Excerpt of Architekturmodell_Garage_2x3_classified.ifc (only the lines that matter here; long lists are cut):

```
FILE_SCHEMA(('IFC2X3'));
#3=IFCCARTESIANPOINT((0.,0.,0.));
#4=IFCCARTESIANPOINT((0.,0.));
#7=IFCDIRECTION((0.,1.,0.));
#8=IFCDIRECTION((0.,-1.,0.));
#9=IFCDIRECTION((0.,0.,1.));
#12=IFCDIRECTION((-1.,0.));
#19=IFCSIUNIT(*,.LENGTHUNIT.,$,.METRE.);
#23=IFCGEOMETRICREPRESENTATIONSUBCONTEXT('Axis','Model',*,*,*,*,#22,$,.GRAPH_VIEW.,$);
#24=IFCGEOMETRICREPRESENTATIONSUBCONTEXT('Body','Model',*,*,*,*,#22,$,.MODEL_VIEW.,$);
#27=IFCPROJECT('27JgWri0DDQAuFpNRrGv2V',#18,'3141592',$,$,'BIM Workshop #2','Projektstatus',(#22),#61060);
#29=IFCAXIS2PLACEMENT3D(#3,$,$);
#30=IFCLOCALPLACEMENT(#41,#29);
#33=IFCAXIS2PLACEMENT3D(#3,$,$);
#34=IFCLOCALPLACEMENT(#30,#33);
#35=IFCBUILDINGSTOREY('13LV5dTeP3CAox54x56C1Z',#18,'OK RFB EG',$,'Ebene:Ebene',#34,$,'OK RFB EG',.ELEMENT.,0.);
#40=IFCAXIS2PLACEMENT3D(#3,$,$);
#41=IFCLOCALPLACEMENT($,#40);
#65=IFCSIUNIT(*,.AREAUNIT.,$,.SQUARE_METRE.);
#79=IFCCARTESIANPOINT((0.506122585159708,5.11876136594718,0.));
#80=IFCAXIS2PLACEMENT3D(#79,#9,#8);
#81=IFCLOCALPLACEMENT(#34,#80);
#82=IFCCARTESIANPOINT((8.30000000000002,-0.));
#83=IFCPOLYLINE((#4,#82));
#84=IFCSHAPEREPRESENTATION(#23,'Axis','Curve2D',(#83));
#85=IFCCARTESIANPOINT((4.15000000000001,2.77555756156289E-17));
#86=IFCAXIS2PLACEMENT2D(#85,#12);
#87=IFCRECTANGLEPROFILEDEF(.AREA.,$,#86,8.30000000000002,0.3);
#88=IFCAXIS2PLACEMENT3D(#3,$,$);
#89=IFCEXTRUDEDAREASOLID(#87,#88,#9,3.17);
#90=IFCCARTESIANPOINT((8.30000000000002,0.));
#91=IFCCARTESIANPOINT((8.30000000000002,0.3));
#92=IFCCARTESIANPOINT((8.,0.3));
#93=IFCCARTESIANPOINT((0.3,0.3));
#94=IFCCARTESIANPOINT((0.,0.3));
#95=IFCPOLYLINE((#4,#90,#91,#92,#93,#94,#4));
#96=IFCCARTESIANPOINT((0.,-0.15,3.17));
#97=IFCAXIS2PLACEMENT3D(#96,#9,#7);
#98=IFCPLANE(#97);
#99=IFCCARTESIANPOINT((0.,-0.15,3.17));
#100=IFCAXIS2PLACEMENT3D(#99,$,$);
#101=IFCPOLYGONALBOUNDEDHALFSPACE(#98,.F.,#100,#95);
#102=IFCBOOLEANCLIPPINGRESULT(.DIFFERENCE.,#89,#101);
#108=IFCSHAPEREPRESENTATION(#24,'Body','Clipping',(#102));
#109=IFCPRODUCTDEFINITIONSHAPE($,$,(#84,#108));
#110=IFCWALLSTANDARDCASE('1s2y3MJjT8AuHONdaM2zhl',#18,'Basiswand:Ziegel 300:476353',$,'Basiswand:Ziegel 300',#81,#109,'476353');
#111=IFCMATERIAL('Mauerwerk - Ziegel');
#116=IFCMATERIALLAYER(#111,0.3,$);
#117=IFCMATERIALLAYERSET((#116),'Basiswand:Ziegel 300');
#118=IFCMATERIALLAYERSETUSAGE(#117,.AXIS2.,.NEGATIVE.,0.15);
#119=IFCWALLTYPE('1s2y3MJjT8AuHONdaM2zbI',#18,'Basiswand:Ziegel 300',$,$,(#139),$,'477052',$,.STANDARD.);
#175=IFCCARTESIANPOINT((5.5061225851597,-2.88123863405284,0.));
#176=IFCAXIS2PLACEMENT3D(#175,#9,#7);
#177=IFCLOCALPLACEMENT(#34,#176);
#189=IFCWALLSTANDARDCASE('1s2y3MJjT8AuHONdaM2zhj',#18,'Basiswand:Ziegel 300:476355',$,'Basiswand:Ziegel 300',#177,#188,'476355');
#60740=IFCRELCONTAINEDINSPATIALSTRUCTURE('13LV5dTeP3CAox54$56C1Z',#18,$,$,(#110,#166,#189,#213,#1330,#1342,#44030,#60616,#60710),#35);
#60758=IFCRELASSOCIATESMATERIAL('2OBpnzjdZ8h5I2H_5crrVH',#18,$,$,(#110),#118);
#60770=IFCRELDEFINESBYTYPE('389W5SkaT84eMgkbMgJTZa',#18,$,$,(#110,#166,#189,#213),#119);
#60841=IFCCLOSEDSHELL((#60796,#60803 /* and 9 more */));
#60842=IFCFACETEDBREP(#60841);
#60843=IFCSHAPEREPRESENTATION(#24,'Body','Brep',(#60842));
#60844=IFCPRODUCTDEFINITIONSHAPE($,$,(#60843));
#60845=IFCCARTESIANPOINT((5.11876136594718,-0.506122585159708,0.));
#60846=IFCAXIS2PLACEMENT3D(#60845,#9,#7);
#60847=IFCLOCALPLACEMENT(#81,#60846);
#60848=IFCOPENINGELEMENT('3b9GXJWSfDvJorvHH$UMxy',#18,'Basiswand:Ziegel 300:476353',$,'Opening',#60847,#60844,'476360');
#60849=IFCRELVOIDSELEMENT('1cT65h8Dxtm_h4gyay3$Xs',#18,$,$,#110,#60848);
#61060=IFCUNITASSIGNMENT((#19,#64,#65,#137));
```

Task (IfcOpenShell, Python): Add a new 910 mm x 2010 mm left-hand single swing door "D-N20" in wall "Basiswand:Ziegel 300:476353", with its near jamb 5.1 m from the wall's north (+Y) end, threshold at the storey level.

```python
import numpy as np
import ifcopenshell
import ifcopenshell.api.feature
import ifcopenshell.api.geometry
import ifcopenshell.api.root
import ifcopenshell.api.spatial
import ifcopenshell.api.type
import ifcopenshell.geom
import ifcopenshell.util.element
import ifcopenshell.util.placement
import ifcopenshell.util.representation
import ifcopenshell.util.shape
import ifcopenshell.util.unit

model = ifcopenshell.open("Architekturmodell_Garage_2x3_classified.ifc")
unit_scale = ifcopenshell.util.unit.calculate_unit_scale(model)
settings = ifcopenshell.geom.settings()


def volume(element):
    """Net volume in cubic metres, openings subtracted."""
    shape = ifcopenshell.geom.create_shape(settings, element)
    return ifcopenshell.util.shape.get_volume(shape.geometry)


wall = model.by_guid("1s2y3MJjT8AuHONdaM2zhl")
storey = ifcopenshell.util.element.get_container(wall, ifc_class="IfcBuildingStorey")
context = ifcopenshell.util.representation.get_context(model, "Model", "Body", "MODEL_VIEW")
before = volume(wall)

width, height, from_end, sill = 0.91, 2.01, 5.1, 0.0  # metres

# The wall runs along its own X axis, and the end named is its -X end.
wall_shape = ifcopenshell.geom.create_shape(settings, wall)
x, y, z = ifcopenshell.util.shape.get_vertices(wall_shape.geometry).T
start = x.min() + from_end
face, thickness = float(y.min()), float(y.max() - y.min())
wall_matrix = ifcopenshell.util.placement.get_local_placement(wall.ObjectPlacement)
level = ifcopenshell.util.placement.get_local_placement(storey.ObjectPlacement)[2, 3]


def in_wall(x, y):
    """Placement at x, y metres in the wall's axes, at sill height."""
    matrix = wall_matrix.copy()
    matrix[:, 3] = wall_matrix @ np.array([x / unit_scale, y / unit_scale, 0.0, 1.0])
    matrix[2, 3] = level + sill / unit_scale
    return matrix


# Opening: a box that overshoots both wall faces by 50 mm.
opening = ifcopenshell.api.root.create_entity(model, ifc_class="IfcOpeningElement")
box = ifcopenshell.api.geometry.add_wall_representation(
    model, context=context, length=width, height=height, thickness=thickness + 0.1
)
ifcopenshell.api.geometry.assign_representation(model, product=opening, representation=box)
ifcopenshell.api.geometry.edit_object_placement(model, product=opening, matrix=in_wall(start, face - 0.05), is_si=False)
ifcopenshell.api.feature.add_feature(model, feature=opening, element=wall)

door = ifcopenshell.api.root.create_entity(model, ifc_class="IfcDoor", name="D-N20")
door.OverallWidth, door.OverallHeight = width / unit_scale, height / unit_scale
body = ifcopenshell.api.geometry.add_door_representation(
    model,
    context=context,
    overall_width=door.OverallWidth,
    overall_height=door.OverallHeight,
    operation_type="SINGLE_SWING_LEFT",
    lining_properties={"LiningDepth": thickness / unit_scale, "ThresholdDepth": thickness / unit_scale},
)
ifcopenshell.api.geometry.assign_representation(model, product=door, representation=body)
ifcopenshell.api.spatial.assign_container(model, products=[door], relating_structure=storey)
fills = ifcopenshell.api.feature.add_filling(model, opening=opening, element=door)
fills.OwnerHistory = door.OwnerHistory  # required in IFC2X3

# IFC2X3 keeps the operation on the door style.
style = ifcopenshell.api.root.create_entity(model, ifc_class="IfcDoorStyle", name="D-N20")
style.OperationType, style.ConstructionType = "SINGLE_SWING_LEFT", "NOTDEFINED"
style.ParameterTakesPrecedence = style.Sizeable = False
ifcopenshell.api.type.assign_type(model, related_objects=[door], relating_type=style)

# The lining spans the wall, so the door starts at the wall face.
ifcopenshell.api.geometry.edit_object_placement(model, product=door, matrix=in_wall(start, face), is_si=False)

after = volume(wall)

print(f"wall volume {before:.3f} -> {after:.3f} m3")

model.write("Architekturmodell_Garage_2x3_classified-out.ifc")
```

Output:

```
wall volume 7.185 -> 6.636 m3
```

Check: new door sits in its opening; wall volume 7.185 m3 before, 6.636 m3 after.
